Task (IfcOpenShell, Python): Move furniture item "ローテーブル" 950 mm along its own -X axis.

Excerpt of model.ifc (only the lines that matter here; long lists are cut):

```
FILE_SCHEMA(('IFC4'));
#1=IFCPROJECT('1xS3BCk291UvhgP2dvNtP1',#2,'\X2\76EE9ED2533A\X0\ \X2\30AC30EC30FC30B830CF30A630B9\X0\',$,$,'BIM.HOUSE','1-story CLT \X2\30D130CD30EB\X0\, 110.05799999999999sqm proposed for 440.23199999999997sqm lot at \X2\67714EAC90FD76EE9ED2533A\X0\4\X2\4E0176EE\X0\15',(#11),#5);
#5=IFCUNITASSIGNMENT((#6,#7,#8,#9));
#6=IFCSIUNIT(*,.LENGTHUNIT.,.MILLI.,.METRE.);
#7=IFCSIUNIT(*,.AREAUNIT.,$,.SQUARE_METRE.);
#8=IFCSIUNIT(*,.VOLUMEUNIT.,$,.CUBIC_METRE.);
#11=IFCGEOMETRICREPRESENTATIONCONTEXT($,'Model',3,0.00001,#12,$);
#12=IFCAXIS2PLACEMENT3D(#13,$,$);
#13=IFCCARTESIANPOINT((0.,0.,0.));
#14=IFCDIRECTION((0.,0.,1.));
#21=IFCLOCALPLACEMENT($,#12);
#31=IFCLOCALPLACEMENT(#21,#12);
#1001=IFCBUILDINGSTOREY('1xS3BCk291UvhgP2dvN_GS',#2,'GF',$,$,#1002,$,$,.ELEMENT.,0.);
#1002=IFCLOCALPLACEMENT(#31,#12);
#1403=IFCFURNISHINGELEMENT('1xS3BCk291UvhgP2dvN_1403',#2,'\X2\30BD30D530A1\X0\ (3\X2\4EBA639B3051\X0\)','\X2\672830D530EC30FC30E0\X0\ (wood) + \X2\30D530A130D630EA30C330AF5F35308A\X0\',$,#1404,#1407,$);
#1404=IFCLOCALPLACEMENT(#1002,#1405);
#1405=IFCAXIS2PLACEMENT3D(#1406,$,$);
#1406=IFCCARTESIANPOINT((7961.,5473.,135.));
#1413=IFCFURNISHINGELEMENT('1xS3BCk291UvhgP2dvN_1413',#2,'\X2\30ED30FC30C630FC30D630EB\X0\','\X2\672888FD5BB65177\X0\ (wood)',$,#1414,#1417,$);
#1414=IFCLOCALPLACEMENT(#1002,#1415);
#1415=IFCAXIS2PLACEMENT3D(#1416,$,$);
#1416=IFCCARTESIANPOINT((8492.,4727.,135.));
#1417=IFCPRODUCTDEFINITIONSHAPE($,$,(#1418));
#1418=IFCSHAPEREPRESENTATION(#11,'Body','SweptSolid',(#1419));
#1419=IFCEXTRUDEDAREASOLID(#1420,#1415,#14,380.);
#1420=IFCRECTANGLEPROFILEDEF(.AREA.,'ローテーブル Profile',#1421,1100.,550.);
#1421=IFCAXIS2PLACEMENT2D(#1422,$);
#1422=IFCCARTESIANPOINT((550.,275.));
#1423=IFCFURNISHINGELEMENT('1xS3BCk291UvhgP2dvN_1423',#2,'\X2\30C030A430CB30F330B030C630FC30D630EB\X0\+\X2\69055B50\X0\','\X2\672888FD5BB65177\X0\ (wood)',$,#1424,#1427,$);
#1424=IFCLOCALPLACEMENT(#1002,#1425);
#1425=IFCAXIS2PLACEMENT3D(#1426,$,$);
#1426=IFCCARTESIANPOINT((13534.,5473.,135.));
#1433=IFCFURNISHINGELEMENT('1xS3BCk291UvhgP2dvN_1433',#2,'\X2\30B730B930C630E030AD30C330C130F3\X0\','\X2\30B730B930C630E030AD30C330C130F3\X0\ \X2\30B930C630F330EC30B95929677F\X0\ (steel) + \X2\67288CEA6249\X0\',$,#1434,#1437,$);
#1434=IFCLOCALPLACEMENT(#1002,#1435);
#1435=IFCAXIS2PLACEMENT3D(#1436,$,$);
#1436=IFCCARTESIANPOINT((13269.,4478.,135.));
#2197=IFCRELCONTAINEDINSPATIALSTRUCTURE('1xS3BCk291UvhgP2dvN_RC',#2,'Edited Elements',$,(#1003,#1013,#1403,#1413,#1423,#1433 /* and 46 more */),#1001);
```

```python
import ifcopenshell
import ifcopenshell.api.geometry
import ifcopenshell.util.placement

model = ifcopenshell.open("model.ifc")

item = model.by_guid("1xS3BCk291UvhgP2dvN_1413")
matrix = ifcopenshell.util.placement.get_local_placement(item.ObjectPlacement)
matrix[:3, 3] -= matrix[:3, 0] * 950.0
ifcopenshell.api.geometry.edit_object_placement(model, product=item, matrix=matrix, is_si=False)

print(ifcopenshell.util.placement.get_local_placement(item.ObjectPlacement).round(3) + 0.0)

model.write("model_rev.ifc")
```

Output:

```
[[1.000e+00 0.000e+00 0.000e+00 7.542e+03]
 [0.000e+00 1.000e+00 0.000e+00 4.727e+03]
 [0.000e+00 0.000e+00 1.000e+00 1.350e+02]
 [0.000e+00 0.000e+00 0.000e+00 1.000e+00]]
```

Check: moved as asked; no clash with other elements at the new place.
